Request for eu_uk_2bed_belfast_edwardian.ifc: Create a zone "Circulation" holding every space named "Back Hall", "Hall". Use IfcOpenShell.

First a look at what the model holds.

```python
import ifcopenshell

model = ifcopenshell.open("eu_uk_2bed_belfast_edwardian.ifc")
print(model.schema)
seen = {}
for space in model.by_type("IfcSpace"):
    seen[space.LongName] = seen.get(space.LongName, 0) + 1
for name, count in sorted(seen.items(), key=str):
    print(count, "x", name)
print("zones:", [z.Name for z in model.by_type("IfcZone")][:20])
```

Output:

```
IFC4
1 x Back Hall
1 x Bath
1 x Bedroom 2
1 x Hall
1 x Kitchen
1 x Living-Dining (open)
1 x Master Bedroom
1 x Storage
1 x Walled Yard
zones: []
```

```python
import ifcopenshell
import ifcopenshell.api.group
import ifcopenshell.api.root

model = ifcopenshell.open("eu_uk_2bed_belfast_edwardian.ifc")

names = {"Back Hall", "Hall"}
spaces = [s for s in model.by_type("IfcSpace") if s.LongName in names]

zone = ifcopenshell.api.root.create_entity(model, ifc_class="IfcZone", name="Circulation")
ifcopenshell.api.group.assign_group(model, products=spaces, group=zone)
print(len(spaces), "spaces in", zone.Name)

model.write("eu_uk_2bed_belfast_edwardian_updated.ifc")
```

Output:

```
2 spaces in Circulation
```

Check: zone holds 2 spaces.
